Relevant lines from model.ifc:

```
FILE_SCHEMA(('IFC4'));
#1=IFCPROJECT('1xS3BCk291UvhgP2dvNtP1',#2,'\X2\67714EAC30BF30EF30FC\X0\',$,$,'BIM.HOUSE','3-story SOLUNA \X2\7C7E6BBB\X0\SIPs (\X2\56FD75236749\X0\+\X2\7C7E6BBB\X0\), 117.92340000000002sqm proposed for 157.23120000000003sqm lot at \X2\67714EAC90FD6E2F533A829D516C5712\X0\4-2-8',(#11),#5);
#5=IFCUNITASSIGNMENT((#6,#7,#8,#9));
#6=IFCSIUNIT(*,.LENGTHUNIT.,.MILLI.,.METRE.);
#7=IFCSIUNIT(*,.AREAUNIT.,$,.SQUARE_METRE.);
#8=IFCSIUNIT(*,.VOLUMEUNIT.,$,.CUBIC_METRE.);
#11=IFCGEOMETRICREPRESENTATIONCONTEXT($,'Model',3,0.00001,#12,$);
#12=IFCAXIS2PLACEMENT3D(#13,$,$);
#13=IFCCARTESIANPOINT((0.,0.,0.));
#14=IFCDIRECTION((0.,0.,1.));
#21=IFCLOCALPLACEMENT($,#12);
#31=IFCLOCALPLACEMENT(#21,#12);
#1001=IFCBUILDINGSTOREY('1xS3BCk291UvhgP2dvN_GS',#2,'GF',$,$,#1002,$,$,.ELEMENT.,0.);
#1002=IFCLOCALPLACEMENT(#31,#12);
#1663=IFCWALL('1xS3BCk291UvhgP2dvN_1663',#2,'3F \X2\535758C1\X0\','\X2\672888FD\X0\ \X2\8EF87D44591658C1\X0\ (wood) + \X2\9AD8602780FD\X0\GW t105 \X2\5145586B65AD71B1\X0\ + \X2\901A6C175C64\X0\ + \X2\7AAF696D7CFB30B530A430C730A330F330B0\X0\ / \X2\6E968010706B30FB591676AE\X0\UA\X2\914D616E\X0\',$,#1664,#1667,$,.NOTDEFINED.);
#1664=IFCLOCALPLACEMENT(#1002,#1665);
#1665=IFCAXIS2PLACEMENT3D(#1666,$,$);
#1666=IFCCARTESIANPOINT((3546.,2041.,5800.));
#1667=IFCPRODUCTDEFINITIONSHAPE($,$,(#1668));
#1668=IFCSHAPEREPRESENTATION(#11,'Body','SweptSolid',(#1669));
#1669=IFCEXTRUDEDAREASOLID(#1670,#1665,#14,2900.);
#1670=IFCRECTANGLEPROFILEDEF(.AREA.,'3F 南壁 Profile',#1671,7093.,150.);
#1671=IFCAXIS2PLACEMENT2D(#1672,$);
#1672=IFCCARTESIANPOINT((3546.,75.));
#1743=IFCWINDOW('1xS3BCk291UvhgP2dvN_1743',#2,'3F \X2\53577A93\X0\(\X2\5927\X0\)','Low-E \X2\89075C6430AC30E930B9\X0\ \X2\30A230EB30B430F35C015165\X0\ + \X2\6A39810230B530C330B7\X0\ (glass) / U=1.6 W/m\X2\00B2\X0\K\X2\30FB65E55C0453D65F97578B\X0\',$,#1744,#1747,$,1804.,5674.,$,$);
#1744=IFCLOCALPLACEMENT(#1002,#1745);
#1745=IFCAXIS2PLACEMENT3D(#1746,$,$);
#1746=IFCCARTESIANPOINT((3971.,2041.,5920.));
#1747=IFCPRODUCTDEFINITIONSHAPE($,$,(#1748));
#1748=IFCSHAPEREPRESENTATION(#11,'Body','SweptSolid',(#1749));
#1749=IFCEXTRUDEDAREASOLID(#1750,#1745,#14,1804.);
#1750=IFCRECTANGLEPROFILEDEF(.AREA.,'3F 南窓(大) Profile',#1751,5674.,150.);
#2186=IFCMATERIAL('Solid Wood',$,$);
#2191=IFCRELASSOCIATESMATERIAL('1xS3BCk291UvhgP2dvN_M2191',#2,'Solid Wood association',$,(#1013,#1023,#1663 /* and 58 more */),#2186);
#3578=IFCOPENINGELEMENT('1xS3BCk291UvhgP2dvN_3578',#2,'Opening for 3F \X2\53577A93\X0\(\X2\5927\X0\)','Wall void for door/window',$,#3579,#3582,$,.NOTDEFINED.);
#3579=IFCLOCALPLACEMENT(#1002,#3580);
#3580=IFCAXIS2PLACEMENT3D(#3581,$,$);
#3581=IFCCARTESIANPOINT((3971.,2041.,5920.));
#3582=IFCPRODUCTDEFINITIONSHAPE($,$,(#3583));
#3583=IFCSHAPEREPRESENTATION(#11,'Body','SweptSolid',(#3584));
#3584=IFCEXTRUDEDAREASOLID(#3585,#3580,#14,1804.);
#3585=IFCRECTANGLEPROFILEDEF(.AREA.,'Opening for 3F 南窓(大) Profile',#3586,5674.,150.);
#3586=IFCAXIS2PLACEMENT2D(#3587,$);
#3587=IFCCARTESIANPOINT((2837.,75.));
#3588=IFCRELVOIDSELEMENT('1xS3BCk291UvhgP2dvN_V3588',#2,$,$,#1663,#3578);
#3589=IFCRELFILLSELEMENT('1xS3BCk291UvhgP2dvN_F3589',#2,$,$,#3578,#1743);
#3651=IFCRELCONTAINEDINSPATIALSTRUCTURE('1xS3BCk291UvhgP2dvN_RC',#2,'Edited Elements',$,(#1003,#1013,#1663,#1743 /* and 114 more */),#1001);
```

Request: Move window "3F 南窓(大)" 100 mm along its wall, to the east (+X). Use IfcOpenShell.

```python
import ifcopenshell
import ifcopenshell.api.geometry
import ifcopenshell.util.placement
import ifcopenshell.util.unit

model = ifcopenshell.open("model.ifc")
unit_scale = ifcopenshell.util.unit.calculate_unit_scale(model)

window = model.by_guid("1xS3BCk291UvhgP2dvN_1743")
opening = window.FillsVoids[0].RelatingOpeningElement
wall = opening.VoidsElements[0].RelatingBuildingElement

wall_matrix = ifcopenshell.util.placement.get_local_placement(wall.ObjectPlacement)
shift = wall_matrix[:3, 0] * 0.1 / unit_scale
before = ifcopenshell.util.placement.get_local_placement(window.ObjectPlacement)[:3, 3].copy()

# The window is not placed relative to its opening, so move both.
for product in (opening, window):
    matrix = ifcopenshell.util.placement.get_local_placement(product.ObjectPlacement)
    matrix[:3, 3] += shift
    ifcopenshell.api.geometry.edit_object_placement(model, product=product, matrix=matrix, is_si=False)

after = ifcopenshell.util.placement.get_local_placement(window.ObjectPlacement)[:3, 3]
print("window moved by", (after - before).round(3) + 0.0)

model.write("model-out.ifc")
```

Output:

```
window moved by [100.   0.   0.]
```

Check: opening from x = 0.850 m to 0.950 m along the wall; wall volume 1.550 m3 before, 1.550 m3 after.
